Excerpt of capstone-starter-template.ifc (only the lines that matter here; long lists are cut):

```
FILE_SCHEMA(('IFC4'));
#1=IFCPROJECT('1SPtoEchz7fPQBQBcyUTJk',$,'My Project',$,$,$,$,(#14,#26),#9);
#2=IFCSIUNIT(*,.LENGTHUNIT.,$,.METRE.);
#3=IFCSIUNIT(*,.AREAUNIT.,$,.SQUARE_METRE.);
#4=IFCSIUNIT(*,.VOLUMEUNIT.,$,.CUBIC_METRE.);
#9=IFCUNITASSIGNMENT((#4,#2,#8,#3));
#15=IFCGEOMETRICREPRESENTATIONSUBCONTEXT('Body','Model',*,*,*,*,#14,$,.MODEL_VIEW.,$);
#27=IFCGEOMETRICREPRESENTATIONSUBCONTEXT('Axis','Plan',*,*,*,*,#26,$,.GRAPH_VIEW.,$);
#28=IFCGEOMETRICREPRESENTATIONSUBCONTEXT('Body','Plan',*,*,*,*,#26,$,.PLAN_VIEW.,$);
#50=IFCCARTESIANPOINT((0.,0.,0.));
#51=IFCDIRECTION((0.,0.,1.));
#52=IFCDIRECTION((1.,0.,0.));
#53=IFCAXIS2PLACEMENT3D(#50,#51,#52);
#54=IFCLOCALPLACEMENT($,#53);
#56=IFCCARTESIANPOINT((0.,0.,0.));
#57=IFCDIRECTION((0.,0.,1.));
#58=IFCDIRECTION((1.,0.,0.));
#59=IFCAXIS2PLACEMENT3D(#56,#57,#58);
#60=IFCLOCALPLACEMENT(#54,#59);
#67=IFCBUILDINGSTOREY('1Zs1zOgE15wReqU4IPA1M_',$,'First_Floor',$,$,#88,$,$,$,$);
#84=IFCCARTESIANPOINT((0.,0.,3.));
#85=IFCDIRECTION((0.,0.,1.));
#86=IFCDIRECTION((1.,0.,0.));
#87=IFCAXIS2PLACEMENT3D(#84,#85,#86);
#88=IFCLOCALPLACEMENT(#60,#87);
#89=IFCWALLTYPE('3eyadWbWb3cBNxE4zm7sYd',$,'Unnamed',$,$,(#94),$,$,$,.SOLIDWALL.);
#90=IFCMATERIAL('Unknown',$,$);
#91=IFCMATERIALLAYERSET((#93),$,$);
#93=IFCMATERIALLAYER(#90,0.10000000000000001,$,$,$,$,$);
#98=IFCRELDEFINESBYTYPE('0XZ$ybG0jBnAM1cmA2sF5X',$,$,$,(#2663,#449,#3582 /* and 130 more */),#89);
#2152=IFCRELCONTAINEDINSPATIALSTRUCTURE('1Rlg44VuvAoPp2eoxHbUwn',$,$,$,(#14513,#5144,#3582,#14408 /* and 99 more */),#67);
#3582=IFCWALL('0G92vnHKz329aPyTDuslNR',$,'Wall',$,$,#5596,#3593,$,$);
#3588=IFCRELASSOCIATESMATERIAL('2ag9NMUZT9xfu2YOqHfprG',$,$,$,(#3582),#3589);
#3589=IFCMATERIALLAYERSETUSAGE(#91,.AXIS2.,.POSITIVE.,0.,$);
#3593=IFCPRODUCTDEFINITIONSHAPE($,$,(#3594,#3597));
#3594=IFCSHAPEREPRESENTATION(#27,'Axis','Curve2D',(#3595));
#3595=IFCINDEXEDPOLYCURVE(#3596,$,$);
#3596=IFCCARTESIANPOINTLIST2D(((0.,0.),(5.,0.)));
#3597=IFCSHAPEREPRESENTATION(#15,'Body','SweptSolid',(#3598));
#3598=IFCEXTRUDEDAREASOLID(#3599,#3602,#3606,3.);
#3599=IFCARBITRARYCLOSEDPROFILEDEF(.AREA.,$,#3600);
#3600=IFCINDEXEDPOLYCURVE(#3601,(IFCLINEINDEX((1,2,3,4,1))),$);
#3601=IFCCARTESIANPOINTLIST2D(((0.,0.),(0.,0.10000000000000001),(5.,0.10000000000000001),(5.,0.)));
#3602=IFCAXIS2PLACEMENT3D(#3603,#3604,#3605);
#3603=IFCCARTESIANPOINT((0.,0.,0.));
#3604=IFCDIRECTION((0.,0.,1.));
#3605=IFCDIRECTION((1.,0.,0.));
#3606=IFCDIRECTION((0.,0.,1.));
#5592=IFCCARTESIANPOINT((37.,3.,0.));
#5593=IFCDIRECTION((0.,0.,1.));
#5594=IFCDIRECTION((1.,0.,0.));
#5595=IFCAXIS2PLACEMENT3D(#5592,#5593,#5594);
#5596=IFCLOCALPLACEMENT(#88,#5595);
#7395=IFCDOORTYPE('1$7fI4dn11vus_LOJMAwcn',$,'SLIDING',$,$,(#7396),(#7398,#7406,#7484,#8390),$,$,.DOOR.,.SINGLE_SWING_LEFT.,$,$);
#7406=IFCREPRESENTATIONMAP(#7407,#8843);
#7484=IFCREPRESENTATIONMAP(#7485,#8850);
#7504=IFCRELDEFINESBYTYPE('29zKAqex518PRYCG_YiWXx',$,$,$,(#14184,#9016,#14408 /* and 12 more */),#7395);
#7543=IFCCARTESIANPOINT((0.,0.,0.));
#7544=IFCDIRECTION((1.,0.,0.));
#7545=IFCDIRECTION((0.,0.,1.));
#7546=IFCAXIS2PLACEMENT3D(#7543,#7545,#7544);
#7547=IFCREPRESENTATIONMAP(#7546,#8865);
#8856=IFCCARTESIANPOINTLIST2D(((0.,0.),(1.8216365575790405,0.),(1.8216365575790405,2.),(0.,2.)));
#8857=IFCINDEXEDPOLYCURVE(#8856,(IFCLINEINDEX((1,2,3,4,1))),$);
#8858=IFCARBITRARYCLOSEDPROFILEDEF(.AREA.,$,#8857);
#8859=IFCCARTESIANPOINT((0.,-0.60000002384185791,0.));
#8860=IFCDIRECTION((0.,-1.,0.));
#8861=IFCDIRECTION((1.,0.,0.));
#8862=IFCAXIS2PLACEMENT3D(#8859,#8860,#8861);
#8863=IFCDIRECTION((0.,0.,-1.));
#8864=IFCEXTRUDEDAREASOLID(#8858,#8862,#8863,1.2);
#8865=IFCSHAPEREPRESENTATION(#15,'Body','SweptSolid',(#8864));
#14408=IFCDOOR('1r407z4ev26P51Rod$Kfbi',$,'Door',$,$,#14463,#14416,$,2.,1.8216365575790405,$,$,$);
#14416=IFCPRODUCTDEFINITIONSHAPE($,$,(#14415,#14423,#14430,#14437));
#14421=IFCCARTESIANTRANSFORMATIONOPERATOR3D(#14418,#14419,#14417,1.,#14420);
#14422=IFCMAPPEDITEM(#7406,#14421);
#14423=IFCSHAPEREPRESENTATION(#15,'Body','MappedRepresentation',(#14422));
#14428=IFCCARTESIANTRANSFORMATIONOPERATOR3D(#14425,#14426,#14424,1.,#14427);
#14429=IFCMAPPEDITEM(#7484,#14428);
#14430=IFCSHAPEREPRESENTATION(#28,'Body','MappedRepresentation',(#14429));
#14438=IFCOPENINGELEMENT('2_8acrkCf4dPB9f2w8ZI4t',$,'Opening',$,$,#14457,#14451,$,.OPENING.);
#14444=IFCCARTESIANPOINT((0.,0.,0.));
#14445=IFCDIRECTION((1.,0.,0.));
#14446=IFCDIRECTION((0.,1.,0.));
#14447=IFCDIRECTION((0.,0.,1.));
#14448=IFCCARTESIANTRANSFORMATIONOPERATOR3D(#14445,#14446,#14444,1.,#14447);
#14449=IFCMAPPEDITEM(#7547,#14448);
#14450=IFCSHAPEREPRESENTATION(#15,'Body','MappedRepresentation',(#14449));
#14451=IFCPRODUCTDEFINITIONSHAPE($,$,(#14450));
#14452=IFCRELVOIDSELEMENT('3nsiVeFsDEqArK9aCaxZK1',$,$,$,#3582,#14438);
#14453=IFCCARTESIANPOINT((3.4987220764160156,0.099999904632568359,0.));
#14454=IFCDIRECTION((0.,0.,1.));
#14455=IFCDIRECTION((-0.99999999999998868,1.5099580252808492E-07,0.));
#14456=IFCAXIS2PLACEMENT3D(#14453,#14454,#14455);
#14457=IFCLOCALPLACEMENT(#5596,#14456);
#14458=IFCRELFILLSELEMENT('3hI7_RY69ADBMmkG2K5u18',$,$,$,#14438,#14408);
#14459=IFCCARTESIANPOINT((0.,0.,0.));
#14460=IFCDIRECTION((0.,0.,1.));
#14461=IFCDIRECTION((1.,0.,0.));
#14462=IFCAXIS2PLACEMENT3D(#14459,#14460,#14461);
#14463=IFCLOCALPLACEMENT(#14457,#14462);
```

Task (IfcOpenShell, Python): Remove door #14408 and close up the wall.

```python
import ifcopenshell
import ifcopenshell.api.feature
import ifcopenshell.api.root
import ifcopenshell.geom
import ifcopenshell.util.shape

model = ifcopenshell.open("capstone-starter-template.ifc")
settings = ifcopenshell.geom.settings()


def volume(element):
    """Net volume in cubic metres, openings subtracted."""
    shape = ifcopenshell.geom.create_shape(settings, element)
    return ifcopenshell.util.shape.get_volume(shape.geometry)


door = model.by_guid("1r407z4ev26P51Rod$Kfbi")
opening = door.FillsVoids[0].RelatingOpeningElement
wall = opening.VoidsElements[0].RelatingBuildingElement
before = volume(wall)

ifcopenshell.api.root.remove_product(model, product=door)
ifcopenshell.api.feature.remove_feature(model, feature=opening)

after = volume(wall)

print(f"wall volume {before:.3f} -> {after:.3f} m3")

model.write("capstone-starter-template-out.ifc")
```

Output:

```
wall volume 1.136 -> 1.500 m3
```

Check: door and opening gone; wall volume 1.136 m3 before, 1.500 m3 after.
